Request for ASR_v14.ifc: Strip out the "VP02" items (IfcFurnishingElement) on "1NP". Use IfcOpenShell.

First a look at what the model holds.

```python
import ifcopenshell
import ifcopenshell.util.element

model = ifcopenshell.open("ASR_v14.ifc")
print(model.schema)
storey = next(s for s in model.by_type("IfcBuildingStorey") if s.Name == "1NP")
furniture = [e for e in ifcopenshell.util.element.get_decomposition(storey) if e.is_a("IfcFurnishingElement")]
seen = {}
for e in furniture:
    element_type = ifcopenshell.util.element.get_type(e)
    name = element_type.Name if element_type not in (None, e) else None
    seen[name] = seen.get(name, 0) + 1
for name, count in sorted(seen.items(), key=str):
    print(count, "x", name)
```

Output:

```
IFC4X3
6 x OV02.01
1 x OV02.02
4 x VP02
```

```python
import ifcopenshell
import ifcopenshell.api.root
import ifcopenshell.util.element

model = ifcopenshell.open("ASR_v14.ifc")

storey = next(s for s in model.by_type("IfcBuildingStorey") if s.Name == "1NP")
furniture = [e for e in ifcopenshell.util.element.get_decomposition(storey) if e.is_a("IfcFurnishingElement")]
targets = [e for e in furniture if (t := ifcopenshell.util.element.get_type(e)) not in (None, e) and t.Name == "VP02"]

for e in targets:
    ifcopenshell.api.root.remove_product(model, product=e)
print(len(targets), "removed")

model.write("ASR_v14_updated.ifc")
```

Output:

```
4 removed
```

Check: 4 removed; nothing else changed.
